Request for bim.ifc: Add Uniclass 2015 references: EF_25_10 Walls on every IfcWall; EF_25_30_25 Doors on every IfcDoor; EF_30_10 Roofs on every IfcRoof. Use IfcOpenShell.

First a look at what the model holds.

```python
import ifcopenshell

model = ifcopenshell.open("bim.ifc")
print(model.schema)
print("classifications:", [c.Name for c in model.by_type("IfcClassification")])
for ifc_class in ("IfcDoor", "IfcRoof", "IfcStair", "IfcWall", "IfcWindow"):
    print(ifc_class, len(model.by_type(ifc_class)))
```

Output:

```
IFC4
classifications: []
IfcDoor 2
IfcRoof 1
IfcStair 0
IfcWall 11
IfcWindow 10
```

```python
import ifcopenshell
import ifcopenshell.api.classification

model = ifcopenshell.open("bim.ifc")

system = ifcopenshell.api.classification.add_classification(model, classification="Uniclass 2015")

codes = {
    "IfcWall": ("EF_25_10", "Walls"),
    "IfcDoor": ("EF_25_30_25", "Doors"),
    "IfcRoof": ("EF_30_10", "Roofs"),
}
for ifc_class, (code, name) in codes.items():
    products = model.by_type(ifc_class)
    ifcopenshell.api.classification.add_reference(
        model, products=products, classification=system, identification=code, name=name
    )
    print(code, len(products))

model.write("bim_v2.ifc")
```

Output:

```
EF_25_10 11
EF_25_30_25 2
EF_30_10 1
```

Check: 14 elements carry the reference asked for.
